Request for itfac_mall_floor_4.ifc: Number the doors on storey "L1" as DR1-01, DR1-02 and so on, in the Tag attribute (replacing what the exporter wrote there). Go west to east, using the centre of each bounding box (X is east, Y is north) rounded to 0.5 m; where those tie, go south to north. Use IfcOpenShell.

First a look at what the model holds.

```python
import ifcopenshell
import ifcopenshell.util.element
import ifcopenshell.util.placement

model = ifcopenshell.open("itfac_mall_floor_4.ifc")
print(model.schema)
storey = next(s for s in model.by_type("IfcBuildingStorey") if s.Name == "L1")
doors = [e for e in ifcopenshell.util.element.get_decomposition(storey) if e.is_a("IfcDoor")]
for e in sorted(doors, key=lambda e: e.id()):
    origin = ifcopenshell.util.placement.get_local_placement(e.ObjectPlacement)[:3, 3]
    print(e.id(), e.Tag, e.Name, origin.round(2) + 0.0, sep=" | ")
```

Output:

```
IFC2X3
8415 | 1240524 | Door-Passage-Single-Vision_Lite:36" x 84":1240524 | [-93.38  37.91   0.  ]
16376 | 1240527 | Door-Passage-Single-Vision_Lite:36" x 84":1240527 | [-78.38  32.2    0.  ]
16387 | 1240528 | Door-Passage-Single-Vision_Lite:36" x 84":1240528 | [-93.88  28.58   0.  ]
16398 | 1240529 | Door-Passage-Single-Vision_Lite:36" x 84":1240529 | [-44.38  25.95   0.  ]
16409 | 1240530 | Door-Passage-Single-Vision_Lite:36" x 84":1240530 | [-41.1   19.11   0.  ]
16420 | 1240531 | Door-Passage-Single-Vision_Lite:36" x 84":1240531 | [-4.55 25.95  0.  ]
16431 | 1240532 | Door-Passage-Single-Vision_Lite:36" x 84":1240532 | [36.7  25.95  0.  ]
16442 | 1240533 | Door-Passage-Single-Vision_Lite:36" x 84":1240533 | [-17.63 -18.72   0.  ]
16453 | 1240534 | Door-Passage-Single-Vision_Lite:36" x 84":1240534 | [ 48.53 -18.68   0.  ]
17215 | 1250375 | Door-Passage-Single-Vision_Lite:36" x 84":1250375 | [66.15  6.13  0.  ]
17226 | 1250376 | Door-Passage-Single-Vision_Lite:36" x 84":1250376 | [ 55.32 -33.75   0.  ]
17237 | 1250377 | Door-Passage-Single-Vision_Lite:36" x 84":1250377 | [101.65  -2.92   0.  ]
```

```python
import ifcopenshell
import ifcopenshell.geom
import ifcopenshell.util.element
import ifcopenshell.util.shape

model = ifcopenshell.open("itfac_mall_floor_4.ifc")
settings = ifcopenshell.geom.settings()
settings.set("use-world-coords", True)


def centre(element):
    shape = ifcopenshell.geom.create_shape(settings, element)
    return ifcopenshell.util.shape.get_bbox_centroid(shape.geometry)


storey = next(s for s in model.by_type("IfcBuildingStorey") if s.Name == "L1")
doors = [e for e in ifcopenshell.util.element.get_decomposition(storey) if e.is_a("IfcDoor")]

# Insertion points can sit at a corner or the storey origin, so sort by the geometry (in metres).
centres = {e: centre(e) for e in doors}
doors.sort(key=lambda e: (round(centres[e][0] / 0.5), centres[e][1]))

for i, e in enumerate(doors, start=1):
    number = f"DR1-{i:02d}"
    e.Tag = number
    print(e.id(), number)

model.write("itfac_mall_floor_4_rev.ifc")
```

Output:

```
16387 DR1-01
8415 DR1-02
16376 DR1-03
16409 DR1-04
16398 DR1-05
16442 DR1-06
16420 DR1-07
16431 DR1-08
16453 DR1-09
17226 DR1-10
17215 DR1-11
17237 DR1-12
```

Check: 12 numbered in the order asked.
